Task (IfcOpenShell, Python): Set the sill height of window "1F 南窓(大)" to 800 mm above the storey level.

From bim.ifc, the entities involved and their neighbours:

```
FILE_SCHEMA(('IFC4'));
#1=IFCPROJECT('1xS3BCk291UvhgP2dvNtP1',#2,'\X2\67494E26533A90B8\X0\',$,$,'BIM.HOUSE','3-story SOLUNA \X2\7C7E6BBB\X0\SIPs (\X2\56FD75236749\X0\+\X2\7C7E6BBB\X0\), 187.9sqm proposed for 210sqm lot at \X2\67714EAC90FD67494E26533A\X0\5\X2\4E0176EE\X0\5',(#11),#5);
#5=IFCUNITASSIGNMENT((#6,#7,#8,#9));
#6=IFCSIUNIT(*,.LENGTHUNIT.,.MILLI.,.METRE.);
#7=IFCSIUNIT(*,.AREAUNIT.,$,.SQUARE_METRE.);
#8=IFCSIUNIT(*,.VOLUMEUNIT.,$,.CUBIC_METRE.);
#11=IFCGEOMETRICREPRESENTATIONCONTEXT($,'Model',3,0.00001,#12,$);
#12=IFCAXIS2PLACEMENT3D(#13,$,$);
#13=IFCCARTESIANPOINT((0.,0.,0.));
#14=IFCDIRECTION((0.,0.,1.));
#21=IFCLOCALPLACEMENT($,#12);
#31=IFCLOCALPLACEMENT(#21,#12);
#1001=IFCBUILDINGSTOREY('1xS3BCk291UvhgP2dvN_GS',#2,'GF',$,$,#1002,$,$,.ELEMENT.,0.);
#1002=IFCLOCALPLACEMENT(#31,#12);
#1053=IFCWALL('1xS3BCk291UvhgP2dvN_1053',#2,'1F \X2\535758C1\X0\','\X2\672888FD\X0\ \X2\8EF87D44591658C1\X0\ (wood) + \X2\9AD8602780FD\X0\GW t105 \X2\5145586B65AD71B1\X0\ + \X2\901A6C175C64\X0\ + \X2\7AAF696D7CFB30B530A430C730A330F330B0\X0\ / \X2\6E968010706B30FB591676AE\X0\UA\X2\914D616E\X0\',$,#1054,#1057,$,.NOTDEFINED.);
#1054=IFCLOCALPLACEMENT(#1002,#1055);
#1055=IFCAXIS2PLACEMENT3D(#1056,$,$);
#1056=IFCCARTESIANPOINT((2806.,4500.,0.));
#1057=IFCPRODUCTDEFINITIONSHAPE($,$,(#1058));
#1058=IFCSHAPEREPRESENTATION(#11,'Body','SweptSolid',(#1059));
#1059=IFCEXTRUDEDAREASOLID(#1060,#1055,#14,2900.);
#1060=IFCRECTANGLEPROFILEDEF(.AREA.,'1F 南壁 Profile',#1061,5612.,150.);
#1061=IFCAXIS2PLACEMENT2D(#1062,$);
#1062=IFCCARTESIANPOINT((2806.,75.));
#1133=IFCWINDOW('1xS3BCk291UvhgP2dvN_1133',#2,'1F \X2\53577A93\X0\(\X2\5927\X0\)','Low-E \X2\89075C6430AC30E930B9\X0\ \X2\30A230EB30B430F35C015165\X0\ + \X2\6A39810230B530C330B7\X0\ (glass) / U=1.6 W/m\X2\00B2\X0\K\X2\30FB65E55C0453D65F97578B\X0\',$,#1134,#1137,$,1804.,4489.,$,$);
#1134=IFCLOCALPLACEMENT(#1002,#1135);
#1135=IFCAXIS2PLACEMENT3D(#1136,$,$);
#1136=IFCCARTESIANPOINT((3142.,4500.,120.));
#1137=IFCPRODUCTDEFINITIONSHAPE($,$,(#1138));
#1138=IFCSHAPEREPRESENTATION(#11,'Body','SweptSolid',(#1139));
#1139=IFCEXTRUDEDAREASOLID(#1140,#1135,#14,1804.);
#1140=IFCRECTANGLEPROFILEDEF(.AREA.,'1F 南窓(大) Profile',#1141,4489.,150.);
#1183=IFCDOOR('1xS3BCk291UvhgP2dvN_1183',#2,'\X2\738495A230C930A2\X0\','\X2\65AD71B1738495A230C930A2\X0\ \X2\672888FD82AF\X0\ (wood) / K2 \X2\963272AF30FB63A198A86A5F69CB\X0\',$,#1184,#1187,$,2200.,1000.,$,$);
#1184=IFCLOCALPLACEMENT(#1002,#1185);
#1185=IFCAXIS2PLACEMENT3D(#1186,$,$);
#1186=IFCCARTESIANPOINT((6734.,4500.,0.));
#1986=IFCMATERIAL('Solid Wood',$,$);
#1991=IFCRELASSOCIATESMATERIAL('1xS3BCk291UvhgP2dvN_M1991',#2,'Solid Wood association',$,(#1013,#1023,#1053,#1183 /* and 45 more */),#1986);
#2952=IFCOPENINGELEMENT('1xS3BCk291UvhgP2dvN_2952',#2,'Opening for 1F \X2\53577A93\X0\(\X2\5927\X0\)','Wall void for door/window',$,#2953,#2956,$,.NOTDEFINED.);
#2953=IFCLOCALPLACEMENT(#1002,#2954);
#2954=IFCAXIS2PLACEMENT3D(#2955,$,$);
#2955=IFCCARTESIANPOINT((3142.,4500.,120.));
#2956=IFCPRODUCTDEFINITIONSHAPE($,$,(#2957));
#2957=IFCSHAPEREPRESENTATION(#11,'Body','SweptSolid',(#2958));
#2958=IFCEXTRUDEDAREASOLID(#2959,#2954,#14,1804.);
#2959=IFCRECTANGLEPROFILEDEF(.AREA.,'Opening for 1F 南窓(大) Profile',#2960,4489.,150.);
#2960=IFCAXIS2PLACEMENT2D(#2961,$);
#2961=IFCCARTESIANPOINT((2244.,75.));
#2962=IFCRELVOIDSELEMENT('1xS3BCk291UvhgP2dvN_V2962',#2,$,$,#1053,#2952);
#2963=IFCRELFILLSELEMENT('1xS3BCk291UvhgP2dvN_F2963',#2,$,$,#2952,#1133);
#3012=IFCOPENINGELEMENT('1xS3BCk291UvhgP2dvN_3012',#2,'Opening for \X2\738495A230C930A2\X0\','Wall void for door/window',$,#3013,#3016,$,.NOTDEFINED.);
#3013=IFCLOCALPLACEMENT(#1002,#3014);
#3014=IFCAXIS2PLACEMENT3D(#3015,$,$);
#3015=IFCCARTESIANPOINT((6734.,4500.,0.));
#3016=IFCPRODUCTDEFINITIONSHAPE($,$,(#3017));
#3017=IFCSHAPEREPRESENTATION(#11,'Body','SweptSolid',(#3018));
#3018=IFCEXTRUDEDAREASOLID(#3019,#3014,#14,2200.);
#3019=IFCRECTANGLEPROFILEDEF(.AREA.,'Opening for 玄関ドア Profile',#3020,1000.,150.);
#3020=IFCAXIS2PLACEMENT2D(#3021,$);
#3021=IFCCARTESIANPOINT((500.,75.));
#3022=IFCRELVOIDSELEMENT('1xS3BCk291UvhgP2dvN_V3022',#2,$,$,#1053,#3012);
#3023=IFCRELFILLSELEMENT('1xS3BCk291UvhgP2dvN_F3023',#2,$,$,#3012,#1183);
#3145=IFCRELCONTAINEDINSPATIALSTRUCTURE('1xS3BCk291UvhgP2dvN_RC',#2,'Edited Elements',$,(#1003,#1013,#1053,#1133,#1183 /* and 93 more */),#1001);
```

```python
import numpy as np
import ifcopenshell
import ifcopenshell.api.geometry
import ifcopenshell.geom
import ifcopenshell.util.element
import ifcopenshell.util.placement
import ifcopenshell.util.shape
import ifcopenshell.util.unit

model = ifcopenshell.open("bim.ifc")
unit_scale = ifcopenshell.util.unit.calculate_unit_scale(model)

window = model.by_id(1133)
opening = window.FillsVoids[0].RelatingOpeningElement
storey = ifcopenshell.util.element.get_container(window, ifc_class="IfcBuildingStorey")
level = ifcopenshell.util.placement.get_local_placement(storey.ObjectPlacement)[2, 3]

# The opening's origin need not be at the sill, so measure its lowest point.
shape = ifcopenshell.geom.create_shape(ifcopenshell.geom.settings(), opening)
bottom = ifcopenshell.util.shape.get_shape_bottom_elevation(shape, shape.geometry) / unit_scale
dz = level + 0.8 / unit_scale - bottom

shift = np.array([0.0, 0.0, dz])
# The window is not placed relative to its opening, so move both.
for product in (opening, window):
    matrix = ifcopenshell.util.placement.get_local_placement(product.ObjectPlacement)
    matrix[:3, 3] += shift
    ifcopenshell.api.geometry.edit_object_placement(model, product=product, matrix=matrix, is_si=False)

print(f"moved by {dz * unit_scale:+.3f} m")

model.write("bim_rev.ifc")
```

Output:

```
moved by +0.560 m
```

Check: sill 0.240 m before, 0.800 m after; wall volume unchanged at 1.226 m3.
